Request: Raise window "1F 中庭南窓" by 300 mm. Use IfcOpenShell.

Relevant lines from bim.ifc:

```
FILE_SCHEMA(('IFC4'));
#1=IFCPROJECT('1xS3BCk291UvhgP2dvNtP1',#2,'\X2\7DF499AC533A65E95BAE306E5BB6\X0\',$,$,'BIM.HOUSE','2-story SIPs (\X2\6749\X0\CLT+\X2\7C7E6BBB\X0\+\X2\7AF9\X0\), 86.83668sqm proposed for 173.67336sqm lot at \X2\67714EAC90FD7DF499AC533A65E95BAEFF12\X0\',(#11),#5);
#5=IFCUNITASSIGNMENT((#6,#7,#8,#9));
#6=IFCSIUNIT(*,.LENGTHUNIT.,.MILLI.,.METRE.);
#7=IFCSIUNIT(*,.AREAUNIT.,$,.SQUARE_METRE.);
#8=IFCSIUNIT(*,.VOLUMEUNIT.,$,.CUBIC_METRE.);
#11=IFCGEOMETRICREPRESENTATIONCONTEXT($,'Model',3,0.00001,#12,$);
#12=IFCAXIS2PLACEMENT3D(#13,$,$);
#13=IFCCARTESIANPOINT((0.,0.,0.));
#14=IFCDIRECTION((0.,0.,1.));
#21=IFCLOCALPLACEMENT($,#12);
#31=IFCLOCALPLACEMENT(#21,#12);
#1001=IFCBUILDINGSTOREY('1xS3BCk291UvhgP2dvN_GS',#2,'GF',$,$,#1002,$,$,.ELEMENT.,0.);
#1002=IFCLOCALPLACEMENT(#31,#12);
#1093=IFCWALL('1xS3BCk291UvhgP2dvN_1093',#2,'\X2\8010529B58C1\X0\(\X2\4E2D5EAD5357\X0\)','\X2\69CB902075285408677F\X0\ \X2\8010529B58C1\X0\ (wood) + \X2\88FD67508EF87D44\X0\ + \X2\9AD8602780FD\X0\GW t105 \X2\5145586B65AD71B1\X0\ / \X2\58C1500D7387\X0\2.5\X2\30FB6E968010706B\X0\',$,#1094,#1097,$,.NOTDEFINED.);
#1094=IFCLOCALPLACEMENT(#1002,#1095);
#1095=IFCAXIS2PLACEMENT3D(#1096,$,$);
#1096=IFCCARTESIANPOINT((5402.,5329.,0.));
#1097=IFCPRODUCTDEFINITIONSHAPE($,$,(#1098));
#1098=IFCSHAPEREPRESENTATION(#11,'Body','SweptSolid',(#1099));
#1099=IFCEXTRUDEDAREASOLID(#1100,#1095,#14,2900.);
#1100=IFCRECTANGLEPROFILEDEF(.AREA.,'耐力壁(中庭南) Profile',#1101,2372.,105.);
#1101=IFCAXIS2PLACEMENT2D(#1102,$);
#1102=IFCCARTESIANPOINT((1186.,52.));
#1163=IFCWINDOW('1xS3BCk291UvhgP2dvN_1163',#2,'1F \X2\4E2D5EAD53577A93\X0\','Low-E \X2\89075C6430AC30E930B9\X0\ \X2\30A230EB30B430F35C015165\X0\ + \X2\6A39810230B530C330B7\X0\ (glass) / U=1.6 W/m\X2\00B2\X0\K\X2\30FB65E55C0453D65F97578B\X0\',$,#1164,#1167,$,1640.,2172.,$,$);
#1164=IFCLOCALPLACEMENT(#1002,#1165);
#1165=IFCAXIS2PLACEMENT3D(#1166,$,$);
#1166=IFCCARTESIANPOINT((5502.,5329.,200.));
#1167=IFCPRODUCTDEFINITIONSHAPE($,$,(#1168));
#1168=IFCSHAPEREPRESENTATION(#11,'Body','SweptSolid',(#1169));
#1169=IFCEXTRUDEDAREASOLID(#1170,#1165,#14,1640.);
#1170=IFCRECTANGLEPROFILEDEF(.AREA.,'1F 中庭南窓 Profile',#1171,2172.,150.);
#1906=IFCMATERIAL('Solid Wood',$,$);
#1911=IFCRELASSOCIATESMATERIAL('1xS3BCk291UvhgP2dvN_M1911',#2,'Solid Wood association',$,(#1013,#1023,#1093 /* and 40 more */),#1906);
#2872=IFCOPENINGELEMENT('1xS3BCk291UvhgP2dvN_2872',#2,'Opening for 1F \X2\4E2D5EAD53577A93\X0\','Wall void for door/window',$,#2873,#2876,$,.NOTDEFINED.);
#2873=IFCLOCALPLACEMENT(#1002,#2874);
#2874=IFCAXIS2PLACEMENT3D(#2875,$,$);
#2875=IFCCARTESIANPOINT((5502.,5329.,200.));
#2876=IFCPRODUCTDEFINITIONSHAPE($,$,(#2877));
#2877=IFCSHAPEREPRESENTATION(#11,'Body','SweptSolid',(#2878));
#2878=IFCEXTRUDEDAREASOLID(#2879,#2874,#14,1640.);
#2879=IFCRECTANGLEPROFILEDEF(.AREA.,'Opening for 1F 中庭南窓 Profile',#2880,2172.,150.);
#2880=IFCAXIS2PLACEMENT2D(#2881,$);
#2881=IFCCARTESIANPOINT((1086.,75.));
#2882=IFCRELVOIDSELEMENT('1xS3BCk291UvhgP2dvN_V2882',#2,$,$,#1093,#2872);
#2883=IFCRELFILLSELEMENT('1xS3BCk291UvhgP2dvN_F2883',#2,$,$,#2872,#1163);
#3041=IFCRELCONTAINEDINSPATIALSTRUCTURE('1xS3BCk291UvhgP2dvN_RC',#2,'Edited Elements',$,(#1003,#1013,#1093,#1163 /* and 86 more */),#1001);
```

```python
import numpy as np
import ifcopenshell
import ifcopenshell.api.geometry
import ifcopenshell.util.placement
import ifcopenshell.util.unit

model = ifcopenshell.open("bim.ifc")
unit_scale = ifcopenshell.util.unit.calculate_unit_scale(model)

window = model.by_id(1163)
opening = window.FillsVoids[0].RelatingOpeningElement
dz = 0.3 / unit_scale

shift = np.array([0.0, 0.0, dz])
# The window is not placed relative to its opening, so move both.
for product in (opening, window):
    matrix = ifcopenshell.util.placement.get_local_placement(product.ObjectPlacement)
    matrix[:3, 3] += shift
    ifcopenshell.api.geometry.edit_object_placement(model, product=product, matrix=matrix, is_si=False)

print(f"moved by {dz * unit_scale:+.3f} m")

model.write("bim_rev.ifc")
```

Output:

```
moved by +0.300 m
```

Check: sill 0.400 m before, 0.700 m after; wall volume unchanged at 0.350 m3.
